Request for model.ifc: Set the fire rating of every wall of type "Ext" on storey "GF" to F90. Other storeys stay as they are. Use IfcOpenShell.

First a look at what the model holds.

```python
import ifcopenshell
import ifcopenshell.util.element

model = ifcopenshell.open("model.ifc")
print(model.schema)
storey = next(s for s in model.by_type("IfcBuildingStorey") if s.Name == "GF")
walls = [e for e in ifcopenshell.util.element.get_decomposition(storey) if e.is_a("IfcWall")]
seen = {}
for e in walls:
    element_type = ifcopenshell.util.element.get_type(e)
    key = (element_type.Name if element_type != e and element_type else None, ifcopenshell.util.element.get_pset(e, "Pset_WallCommon", "FireRating"))
    seen[key] = seen.get(key, 0) + 1
for (name, value), count in sorted(seen.items(), key=str):
    print(count, "x", name, "|", value)
```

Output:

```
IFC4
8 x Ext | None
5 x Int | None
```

```python
import ifcopenshell
import ifcopenshell.api.pset
import ifcopenshell.util.element

model = ifcopenshell.open("model.ifc")

storey = next(s for s in model.by_type("IfcBuildingStorey") if s.Name == "GF")
walls = [e for e in ifcopenshell.util.element.get_decomposition(storey) if e.is_a("IfcWall")]

count = 0
for e in walls:
    element_type = ifcopenshell.util.element.get_type(e)
    if element_type in (None, e) or element_type.Name != "Ext":
        continue
    # add_pset returns the element's existing set when there is one.
    pset = ifcopenshell.api.pset.add_pset(model, product=e, name="Pset_WallCommon")
    ifcopenshell.api.pset.edit_pset(model, pset=pset, properties={"FireRating": "F90"})
    count += 1

print(count, "walls updated")

model.write("model_updated.ifc")
```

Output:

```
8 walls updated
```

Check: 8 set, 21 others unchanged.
